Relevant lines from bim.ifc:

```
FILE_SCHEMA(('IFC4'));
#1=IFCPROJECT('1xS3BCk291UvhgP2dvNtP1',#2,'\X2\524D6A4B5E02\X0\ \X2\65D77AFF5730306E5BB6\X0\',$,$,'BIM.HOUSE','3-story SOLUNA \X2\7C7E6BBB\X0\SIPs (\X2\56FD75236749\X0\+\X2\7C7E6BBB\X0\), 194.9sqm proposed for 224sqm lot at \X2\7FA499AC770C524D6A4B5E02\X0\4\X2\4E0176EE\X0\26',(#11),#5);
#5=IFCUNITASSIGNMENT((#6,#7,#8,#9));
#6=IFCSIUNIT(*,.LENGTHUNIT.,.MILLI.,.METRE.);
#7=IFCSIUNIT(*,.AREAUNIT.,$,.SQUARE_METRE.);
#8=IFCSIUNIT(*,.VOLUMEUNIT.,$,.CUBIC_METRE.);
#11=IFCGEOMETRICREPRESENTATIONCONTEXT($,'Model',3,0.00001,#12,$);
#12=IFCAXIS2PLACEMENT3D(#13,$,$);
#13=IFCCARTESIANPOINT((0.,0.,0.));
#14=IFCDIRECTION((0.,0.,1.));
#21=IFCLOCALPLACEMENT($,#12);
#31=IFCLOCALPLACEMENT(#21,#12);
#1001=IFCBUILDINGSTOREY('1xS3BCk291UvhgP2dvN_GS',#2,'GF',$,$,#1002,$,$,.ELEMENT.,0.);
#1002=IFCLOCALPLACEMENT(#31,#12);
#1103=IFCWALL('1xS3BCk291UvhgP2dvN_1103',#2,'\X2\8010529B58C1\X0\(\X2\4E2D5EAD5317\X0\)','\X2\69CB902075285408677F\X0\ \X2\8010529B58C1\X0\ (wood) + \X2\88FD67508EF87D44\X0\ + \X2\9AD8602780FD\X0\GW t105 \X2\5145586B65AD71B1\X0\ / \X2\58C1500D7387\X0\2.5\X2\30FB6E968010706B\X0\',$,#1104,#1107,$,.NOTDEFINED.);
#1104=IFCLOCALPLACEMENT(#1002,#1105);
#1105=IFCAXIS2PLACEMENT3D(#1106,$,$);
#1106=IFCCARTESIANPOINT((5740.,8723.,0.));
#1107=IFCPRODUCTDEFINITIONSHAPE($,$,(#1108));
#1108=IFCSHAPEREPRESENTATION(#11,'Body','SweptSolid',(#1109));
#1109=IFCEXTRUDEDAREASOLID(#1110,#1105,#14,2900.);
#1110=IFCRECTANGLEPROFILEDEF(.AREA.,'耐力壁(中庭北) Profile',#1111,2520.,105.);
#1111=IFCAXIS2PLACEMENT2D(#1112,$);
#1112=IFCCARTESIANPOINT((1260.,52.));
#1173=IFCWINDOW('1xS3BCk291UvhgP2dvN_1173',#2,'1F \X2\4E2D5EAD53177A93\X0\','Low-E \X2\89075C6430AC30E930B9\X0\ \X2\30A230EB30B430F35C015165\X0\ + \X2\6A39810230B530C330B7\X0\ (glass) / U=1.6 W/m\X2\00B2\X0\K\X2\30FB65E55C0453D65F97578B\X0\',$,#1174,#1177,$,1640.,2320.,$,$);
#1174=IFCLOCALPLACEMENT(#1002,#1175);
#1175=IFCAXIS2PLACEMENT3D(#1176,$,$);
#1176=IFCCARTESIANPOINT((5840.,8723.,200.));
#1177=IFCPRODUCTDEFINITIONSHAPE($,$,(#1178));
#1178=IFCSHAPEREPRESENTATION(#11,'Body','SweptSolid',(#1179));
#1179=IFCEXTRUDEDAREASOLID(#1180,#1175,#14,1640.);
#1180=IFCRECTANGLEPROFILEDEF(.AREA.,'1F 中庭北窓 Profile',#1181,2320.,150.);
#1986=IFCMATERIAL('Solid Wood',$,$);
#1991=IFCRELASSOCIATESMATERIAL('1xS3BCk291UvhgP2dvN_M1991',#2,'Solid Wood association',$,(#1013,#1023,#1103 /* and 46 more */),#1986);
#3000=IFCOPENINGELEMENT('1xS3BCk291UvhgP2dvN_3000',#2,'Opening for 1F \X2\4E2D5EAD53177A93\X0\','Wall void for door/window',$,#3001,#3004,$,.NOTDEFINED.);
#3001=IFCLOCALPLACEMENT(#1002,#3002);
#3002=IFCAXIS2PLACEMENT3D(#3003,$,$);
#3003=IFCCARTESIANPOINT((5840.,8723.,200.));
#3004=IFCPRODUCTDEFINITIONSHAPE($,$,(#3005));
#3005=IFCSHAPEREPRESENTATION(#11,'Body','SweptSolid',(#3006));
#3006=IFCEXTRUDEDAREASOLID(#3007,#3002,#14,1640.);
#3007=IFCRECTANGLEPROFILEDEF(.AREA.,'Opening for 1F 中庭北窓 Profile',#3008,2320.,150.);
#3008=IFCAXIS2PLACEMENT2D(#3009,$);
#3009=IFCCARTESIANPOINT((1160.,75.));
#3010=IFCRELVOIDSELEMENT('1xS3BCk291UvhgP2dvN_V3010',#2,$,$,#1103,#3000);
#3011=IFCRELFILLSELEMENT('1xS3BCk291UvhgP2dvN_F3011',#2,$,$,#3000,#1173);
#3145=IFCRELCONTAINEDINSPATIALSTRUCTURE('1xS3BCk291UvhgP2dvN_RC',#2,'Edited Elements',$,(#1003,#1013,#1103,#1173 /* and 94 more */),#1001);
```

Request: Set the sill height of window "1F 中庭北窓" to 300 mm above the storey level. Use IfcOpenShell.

```python
import numpy as np
import ifcopenshell
import ifcopenshell.api.geometry
import ifcopenshell.geom
import ifcopenshell.util.element
import ifcopenshell.util.placement
import ifcopenshell.util.shape
import ifcopenshell.util.unit

model = ifcopenshell.open("bim.ifc")
unit_scale = ifcopenshell.util.unit.calculate_unit_scale(model)

window = model.by_guid("1xS3BCk291UvhgP2dvN_1173")
opening = window.FillsVoids[0].RelatingOpeningElement
storey = ifcopenshell.util.element.get_container(window, ifc_class="IfcBuildingStorey")
level = ifcopenshell.util.placement.get_local_placement(storey.ObjectPlacement)[2, 3]

# The opening's origin need not be at the sill, so measure its lowest point.
shape = ifcopenshell.geom.create_shape(ifcopenshell.geom.settings(), opening)
bottom = ifcopenshell.util.shape.get_shape_bottom_elevation(shape, shape.geometry) / unit_scale
dz = level + 0.3 / unit_scale - bottom

shift = np.array([0.0, 0.0, dz])
# The window is not placed relative to its opening, so move both.
for product in (opening, window):
    matrix = ifcopenshell.util.placement.get_local_placement(product.ObjectPlacement)
    matrix[:3, 3] += shift
    ifcopenshell.api.geometry.edit_object_placement(model, product=product, matrix=matrix, is_si=False)

print(f"moved by {dz * unit_scale:+.3f} m")

model.write("bim_rev.ifc")
```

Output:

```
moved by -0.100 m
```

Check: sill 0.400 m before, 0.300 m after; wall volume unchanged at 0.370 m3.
